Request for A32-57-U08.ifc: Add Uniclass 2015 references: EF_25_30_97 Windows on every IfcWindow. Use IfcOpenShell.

First a look at what the model holds.

```python
import ifcopenshell

model = ifcopenshell.open("A32-57-U08.ifc")
print(model.schema)
print("classifications:", [c.Name for c in model.by_type("IfcClassification")])
for ifc_class in ("IfcDoor", "IfcRoof", "IfcStair", "IfcWall", "IfcWindow"):
    print(ifc_class, len(model.by_type(ifc_class)))
```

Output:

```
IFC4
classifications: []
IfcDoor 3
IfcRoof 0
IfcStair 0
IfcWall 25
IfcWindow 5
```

```python
import ifcopenshell
import ifcopenshell.api.classification

model = ifcopenshell.open("A32-57-U08.ifc")

system = ifcopenshell.api.classification.add_classification(model, classification="Uniclass 2015")

codes = {
    "IfcWindow": ("EF_25_30_97", "Windows"),
}
for ifc_class, (code, name) in codes.items():
    products = model.by_type(ifc_class)
    ifcopenshell.api.classification.add_reference(
        model, products=products, classification=system, identification=code, name=name
    )
    print(code, len(products))

model.write("A32-57-U08_edited.ifc")
```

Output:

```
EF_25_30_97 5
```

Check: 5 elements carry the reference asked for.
